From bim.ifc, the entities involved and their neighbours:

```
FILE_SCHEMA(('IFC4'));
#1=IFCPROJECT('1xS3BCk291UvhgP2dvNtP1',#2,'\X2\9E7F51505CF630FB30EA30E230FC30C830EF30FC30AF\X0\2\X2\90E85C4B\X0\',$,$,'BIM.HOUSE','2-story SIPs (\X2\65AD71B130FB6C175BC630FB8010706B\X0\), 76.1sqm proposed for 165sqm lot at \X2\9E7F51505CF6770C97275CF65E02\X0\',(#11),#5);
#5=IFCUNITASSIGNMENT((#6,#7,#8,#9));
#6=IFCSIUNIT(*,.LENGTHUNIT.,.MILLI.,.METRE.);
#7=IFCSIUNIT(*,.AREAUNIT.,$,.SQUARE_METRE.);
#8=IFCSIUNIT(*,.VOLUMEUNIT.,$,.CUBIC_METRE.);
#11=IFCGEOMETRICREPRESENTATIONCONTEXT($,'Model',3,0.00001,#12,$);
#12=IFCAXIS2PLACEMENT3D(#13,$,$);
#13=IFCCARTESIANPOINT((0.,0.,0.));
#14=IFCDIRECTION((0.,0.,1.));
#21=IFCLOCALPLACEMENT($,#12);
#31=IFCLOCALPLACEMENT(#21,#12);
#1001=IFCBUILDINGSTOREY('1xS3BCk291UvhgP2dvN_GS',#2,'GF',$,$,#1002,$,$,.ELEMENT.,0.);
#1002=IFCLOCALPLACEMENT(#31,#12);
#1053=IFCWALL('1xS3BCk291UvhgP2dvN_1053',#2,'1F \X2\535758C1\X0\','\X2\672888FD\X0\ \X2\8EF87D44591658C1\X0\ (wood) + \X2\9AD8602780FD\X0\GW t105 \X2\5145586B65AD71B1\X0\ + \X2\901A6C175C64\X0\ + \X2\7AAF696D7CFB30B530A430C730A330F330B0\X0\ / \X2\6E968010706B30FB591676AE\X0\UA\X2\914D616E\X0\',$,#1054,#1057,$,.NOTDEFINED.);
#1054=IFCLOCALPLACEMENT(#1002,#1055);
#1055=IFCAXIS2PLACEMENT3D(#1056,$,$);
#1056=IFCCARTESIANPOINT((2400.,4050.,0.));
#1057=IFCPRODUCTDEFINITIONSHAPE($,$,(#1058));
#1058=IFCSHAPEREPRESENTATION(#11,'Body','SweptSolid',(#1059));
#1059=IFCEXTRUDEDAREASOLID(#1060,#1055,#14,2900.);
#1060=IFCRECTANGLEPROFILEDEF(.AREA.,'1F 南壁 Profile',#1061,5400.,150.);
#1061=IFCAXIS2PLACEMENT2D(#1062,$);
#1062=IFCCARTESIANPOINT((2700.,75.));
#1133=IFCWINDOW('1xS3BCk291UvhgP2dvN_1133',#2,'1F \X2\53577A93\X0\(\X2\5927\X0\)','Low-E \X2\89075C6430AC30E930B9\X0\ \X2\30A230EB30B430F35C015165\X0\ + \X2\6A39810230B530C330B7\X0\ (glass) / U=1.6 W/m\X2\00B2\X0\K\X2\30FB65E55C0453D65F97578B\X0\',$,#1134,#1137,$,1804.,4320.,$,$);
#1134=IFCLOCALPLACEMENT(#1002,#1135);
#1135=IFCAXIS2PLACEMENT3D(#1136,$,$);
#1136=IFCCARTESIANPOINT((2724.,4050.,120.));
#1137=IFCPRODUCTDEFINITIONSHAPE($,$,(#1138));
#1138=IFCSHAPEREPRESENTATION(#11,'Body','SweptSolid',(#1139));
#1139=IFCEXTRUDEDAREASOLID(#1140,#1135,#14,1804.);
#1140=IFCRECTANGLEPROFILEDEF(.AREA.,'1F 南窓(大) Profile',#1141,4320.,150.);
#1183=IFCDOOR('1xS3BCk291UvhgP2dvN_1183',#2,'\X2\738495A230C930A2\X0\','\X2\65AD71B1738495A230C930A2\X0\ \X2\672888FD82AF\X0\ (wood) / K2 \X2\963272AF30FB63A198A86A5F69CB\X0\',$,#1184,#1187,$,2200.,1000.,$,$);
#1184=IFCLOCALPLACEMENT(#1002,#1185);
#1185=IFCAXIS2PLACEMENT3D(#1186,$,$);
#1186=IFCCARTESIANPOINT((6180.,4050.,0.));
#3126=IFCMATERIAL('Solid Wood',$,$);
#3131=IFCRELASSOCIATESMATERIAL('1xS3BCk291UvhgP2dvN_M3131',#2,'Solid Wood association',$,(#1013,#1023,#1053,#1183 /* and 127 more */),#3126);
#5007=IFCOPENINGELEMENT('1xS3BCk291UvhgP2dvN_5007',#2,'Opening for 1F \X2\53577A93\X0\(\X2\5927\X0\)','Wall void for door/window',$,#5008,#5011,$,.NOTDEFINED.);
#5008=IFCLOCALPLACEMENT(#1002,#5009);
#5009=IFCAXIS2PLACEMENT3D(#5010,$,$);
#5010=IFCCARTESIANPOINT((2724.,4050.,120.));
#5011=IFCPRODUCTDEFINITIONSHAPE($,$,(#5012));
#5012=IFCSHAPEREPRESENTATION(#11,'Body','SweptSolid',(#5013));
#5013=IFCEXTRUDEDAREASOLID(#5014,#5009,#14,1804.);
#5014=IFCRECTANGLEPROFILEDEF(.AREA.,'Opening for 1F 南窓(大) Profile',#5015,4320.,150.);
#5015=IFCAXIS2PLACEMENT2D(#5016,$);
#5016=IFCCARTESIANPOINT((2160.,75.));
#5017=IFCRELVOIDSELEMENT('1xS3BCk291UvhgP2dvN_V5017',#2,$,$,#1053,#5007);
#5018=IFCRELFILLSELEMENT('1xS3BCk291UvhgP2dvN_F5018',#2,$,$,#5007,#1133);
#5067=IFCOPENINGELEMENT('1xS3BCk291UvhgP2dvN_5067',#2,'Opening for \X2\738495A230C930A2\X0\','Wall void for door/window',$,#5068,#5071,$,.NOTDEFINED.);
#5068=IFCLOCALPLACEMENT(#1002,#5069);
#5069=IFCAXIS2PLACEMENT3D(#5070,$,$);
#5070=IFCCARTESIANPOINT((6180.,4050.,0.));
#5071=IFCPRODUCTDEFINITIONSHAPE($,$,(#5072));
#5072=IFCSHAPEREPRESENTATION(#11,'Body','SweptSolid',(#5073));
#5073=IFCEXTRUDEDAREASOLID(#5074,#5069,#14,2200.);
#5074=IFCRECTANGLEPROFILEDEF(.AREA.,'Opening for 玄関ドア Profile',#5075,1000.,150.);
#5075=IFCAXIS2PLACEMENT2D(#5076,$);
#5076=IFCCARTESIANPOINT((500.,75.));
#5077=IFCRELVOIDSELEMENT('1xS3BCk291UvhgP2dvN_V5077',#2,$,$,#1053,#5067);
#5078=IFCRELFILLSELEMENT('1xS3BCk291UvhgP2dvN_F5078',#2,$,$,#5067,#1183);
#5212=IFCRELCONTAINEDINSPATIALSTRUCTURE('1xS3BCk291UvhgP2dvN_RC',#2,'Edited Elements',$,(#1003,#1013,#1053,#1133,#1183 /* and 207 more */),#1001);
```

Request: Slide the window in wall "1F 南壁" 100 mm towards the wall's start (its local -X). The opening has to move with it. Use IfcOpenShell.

```python
import ifcopenshell
import ifcopenshell.api.geometry
import ifcopenshell.util.placement

model = ifcopenshell.open("bim.ifc")

window = model.by_guid("1xS3BCk291UvhgP2dvN_1133")
opening = window.FillsVoids[0].RelatingOpeningElement
wall = opening.VoidsElements[0].RelatingBuildingElement

wall_matrix = ifcopenshell.util.placement.get_local_placement(wall.ObjectPlacement)
shift = wall_matrix[:3, 0] * -100.0
before = ifcopenshell.util.placement.get_local_placement(window.ObjectPlacement)[:3, 3].copy()

# The window is not placed relative to its opening, so move both.
for product in (opening, window):
    matrix = ifcopenshell.util.placement.get_local_placement(product.ObjectPlacement)
    matrix[:3, 3] += shift
    ifcopenshell.api.geometry.edit_object_placement(model, product=product, matrix=matrix, is_si=False)

after = ifcopenshell.util.placement.get_local_placement(window.ObjectPlacement)[:3, 3]
print("window moved by", (after - before).round(3) + 0.0)

model.write("bim_rev.ifc")
```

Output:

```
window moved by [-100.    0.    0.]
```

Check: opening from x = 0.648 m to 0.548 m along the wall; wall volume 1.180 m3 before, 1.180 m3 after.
